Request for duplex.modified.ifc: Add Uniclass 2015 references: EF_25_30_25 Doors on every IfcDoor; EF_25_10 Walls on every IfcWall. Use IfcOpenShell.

First a look at what the model holds.

```python
import ifcopenshell

model = ifcopenshell.open("duplex.modified.ifc")
print(model.schema)
print("classifications:", [c.Name for c in model.by_type("IfcClassification")])
for ifc_class in ("IfcDoor", "IfcRoof", "IfcStair", "IfcWall", "IfcWindow"):
    print(ifc_class, len(model.by_type(ifc_class)))
```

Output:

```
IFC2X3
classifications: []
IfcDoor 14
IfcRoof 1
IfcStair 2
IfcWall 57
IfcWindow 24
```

```python
import ifcopenshell
import ifcopenshell.api.classification

model = ifcopenshell.open("duplex.modified.ifc")

# IFC2X3 requires Source and Edition and has no link from the project to the system.
system = model.create_entity("IfcClassification", Source="NBS", Edition="2015", Name="Uniclass 2015")

codes = {
    "IfcDoor": ("EF_25_30_25", "Doors"),
    "IfcWall": ("EF_25_10", "Walls"),
}
for ifc_class, (code, name) in codes.items():
    products = model.by_type(ifc_class)
    ifcopenshell.api.classification.add_reference(
        model, products=products, classification=system, identification=code, name=name
    )
    print(code, len(products))

model.write("duplex.modified_v2.ifc")
```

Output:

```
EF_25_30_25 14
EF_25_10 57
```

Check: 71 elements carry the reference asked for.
